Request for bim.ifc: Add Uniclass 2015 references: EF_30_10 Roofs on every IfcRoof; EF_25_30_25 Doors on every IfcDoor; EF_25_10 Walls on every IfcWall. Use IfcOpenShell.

First a look at what the model holds.

```python
import ifcopenshell

model = ifcopenshell.open("bim.ifc")
print(model.schema)
print("classifications:", [c.Name for c in model.by_type("IfcClassification")])
for ifc_class in ("IfcDoor", "IfcRoof", "IfcStair", "IfcWall", "IfcWindow"):
    print(ifc_class, len(model.by_type(ifc_class)))
```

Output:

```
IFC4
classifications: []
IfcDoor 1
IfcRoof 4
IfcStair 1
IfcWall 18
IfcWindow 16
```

```python
import ifcopenshell
import ifcopenshell.api.classification

model = ifcopenshell.open("bim.ifc")

system = ifcopenshell.api.classification.add_classification(model, classification="Uniclass 2015")

codes = {
    "IfcRoof": ("EF_30_10", "Roofs"),
    "IfcDoor": ("EF_25_30_25", "Doors"),
    "IfcWall": ("EF_25_10", "Walls"),
}
for ifc_class, (code, name) in codes.items():
    products = model.by_type(ifc_class)
    ifcopenshell.api.classification.add_reference(
        model, products=products, classification=system, identification=code, name=name
    )
    print(code, len(products))

model.write("bim_edited.ifc")
```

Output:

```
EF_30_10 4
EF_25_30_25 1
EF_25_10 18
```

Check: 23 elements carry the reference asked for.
